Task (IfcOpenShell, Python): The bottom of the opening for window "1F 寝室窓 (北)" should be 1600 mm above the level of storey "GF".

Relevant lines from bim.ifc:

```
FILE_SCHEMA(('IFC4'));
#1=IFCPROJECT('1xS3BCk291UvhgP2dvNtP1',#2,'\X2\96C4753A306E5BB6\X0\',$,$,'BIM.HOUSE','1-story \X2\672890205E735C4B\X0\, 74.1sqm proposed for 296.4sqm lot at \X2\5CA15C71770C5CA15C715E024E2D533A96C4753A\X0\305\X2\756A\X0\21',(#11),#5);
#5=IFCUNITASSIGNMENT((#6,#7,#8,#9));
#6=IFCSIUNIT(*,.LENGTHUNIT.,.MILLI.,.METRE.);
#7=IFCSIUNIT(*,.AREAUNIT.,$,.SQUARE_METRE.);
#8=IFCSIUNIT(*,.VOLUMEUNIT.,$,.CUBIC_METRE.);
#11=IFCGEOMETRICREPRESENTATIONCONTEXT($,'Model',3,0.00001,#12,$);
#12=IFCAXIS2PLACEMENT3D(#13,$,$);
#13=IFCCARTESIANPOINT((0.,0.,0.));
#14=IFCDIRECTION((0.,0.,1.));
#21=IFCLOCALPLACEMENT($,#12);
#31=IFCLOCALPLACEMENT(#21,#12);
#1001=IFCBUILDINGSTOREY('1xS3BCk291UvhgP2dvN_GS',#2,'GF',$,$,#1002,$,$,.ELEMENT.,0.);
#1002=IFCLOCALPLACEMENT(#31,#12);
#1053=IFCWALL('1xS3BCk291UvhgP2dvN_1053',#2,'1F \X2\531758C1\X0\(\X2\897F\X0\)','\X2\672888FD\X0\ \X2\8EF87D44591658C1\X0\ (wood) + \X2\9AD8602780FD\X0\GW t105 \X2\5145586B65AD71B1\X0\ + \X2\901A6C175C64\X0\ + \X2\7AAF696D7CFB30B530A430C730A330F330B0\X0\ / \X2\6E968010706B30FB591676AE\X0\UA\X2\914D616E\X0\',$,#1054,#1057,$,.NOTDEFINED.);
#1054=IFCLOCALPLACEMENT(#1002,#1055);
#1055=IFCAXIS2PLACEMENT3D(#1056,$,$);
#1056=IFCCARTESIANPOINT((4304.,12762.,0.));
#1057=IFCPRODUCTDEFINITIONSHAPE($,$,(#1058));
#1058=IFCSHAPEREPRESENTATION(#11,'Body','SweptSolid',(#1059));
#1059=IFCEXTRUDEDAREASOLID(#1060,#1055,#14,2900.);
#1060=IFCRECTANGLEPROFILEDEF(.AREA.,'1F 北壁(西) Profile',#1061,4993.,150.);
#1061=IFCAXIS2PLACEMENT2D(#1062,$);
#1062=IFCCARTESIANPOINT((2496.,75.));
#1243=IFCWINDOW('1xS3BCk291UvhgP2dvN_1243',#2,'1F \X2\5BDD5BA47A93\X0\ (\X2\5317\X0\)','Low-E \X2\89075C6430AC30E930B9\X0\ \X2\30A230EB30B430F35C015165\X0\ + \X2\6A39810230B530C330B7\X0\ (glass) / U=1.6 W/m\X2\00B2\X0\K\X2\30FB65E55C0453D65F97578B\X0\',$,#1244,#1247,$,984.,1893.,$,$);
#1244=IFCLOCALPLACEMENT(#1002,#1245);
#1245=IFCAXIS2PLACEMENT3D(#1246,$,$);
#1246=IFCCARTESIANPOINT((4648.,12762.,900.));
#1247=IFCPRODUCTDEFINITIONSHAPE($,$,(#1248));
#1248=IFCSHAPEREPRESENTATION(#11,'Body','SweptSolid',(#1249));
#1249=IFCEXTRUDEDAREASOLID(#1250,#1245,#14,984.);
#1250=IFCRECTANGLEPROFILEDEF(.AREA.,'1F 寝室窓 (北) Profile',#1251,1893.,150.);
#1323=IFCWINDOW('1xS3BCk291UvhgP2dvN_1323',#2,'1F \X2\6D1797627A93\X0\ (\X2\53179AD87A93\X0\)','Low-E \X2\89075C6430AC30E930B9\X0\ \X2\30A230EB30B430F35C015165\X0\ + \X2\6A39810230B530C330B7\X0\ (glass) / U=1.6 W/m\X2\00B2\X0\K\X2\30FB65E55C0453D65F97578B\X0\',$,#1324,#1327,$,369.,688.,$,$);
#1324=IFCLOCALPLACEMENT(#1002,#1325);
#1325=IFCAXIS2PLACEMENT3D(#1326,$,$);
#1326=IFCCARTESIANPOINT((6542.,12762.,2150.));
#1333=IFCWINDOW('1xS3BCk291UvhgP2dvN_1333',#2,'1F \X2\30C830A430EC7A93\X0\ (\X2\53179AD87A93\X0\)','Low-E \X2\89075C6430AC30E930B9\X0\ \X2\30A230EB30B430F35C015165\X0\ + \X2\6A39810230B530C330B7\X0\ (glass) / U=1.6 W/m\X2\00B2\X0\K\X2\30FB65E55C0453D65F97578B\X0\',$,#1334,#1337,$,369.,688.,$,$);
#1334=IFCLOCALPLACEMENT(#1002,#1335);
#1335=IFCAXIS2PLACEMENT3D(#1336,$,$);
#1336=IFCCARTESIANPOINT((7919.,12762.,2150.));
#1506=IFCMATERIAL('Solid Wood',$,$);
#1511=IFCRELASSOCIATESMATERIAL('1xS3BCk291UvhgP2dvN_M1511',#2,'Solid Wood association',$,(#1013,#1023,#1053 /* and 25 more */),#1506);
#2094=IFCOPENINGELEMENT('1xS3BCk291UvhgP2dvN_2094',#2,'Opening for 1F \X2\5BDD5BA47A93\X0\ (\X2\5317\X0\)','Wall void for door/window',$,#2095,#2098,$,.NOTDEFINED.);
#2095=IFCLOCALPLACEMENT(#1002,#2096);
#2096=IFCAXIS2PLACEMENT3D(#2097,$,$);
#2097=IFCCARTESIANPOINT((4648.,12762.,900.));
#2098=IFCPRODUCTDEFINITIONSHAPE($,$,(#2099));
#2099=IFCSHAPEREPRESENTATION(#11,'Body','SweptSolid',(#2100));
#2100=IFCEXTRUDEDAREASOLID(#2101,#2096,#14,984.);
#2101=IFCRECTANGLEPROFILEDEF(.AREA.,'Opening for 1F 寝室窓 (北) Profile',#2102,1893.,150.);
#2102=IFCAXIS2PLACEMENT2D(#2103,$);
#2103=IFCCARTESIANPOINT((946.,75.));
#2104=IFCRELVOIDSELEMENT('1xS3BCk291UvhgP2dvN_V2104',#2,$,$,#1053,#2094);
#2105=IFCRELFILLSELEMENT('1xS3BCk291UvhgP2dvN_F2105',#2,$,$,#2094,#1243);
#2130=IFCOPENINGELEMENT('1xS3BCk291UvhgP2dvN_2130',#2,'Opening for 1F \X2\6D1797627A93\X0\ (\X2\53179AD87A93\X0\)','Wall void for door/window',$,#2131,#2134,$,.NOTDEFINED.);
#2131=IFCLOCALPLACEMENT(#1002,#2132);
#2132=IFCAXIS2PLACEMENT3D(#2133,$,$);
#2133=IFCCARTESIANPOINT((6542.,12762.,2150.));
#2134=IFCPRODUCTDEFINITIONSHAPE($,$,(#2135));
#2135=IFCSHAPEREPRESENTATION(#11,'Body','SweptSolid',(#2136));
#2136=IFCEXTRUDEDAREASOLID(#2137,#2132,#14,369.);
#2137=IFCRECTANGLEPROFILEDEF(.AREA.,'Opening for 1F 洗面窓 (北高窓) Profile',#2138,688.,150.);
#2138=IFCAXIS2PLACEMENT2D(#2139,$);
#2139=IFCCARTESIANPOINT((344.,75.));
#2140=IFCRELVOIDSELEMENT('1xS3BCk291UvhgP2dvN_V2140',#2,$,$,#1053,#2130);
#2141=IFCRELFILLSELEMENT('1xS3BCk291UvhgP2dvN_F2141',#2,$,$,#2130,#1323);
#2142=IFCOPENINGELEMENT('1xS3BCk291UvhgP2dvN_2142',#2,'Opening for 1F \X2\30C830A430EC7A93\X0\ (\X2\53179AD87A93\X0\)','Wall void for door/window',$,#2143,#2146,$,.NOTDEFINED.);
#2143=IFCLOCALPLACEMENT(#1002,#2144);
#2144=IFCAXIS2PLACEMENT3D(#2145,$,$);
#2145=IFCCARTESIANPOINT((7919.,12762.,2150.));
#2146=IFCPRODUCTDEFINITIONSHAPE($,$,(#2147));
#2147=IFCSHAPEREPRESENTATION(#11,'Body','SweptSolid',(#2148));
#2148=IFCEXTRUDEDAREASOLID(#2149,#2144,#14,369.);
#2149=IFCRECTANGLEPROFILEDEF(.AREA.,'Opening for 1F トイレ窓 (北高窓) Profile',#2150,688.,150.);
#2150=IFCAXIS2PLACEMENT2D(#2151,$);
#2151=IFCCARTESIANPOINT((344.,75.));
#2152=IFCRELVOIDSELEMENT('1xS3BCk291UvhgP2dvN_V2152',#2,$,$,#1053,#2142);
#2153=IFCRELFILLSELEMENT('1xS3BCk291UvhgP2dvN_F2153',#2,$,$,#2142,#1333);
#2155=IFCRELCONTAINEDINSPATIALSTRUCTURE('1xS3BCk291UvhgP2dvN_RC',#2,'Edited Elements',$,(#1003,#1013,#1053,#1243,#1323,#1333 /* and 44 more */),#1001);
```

```python
import numpy as np
import ifcopenshell
import ifcopenshell.api.geometry
import ifcopenshell.geom
import ifcopenshell.util.element
import ifcopenshell.util.placement
import ifcopenshell.util.shape
import ifcopenshell.util.unit

model = ifcopenshell.open("bim.ifc")
unit_scale = ifcopenshell.util.unit.calculate_unit_scale(model)

window = model.by_guid("1xS3BCk291UvhgP2dvN_1243")
opening = window.FillsVoids[0].RelatingOpeningElement
storey = ifcopenshell.util.element.get_container(window, ifc_class="IfcBuildingStorey")
level = ifcopenshell.util.placement.get_local_placement(storey.ObjectPlacement)[2, 3]

# The opening's origin need not be at the sill, so measure its lowest point.
shape = ifcopenshell.geom.create_shape(ifcopenshell.geom.settings(), opening)
bottom = ifcopenshell.util.shape.get_shape_bottom_elevation(shape, shape.geometry) / unit_scale
dz = level + 1.6 / unit_scale - bottom

shift = np.array([0.0, 0.0, dz])
# The window is not placed relative to its opening, so move both.
for product in (opening, window):
    matrix = ifcopenshell.util.placement.get_local_placement(product.ObjectPlacement)
    matrix[:3, 3] += shift
    ifcopenshell.api.geometry.edit_object_placement(model, product=product, matrix=matrix, is_si=False)

print(f"moved by {dz * unit_scale:+.3f} m")

model.write("bim_rev.ifc")
```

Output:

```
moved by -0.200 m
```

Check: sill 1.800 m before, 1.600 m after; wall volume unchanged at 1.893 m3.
